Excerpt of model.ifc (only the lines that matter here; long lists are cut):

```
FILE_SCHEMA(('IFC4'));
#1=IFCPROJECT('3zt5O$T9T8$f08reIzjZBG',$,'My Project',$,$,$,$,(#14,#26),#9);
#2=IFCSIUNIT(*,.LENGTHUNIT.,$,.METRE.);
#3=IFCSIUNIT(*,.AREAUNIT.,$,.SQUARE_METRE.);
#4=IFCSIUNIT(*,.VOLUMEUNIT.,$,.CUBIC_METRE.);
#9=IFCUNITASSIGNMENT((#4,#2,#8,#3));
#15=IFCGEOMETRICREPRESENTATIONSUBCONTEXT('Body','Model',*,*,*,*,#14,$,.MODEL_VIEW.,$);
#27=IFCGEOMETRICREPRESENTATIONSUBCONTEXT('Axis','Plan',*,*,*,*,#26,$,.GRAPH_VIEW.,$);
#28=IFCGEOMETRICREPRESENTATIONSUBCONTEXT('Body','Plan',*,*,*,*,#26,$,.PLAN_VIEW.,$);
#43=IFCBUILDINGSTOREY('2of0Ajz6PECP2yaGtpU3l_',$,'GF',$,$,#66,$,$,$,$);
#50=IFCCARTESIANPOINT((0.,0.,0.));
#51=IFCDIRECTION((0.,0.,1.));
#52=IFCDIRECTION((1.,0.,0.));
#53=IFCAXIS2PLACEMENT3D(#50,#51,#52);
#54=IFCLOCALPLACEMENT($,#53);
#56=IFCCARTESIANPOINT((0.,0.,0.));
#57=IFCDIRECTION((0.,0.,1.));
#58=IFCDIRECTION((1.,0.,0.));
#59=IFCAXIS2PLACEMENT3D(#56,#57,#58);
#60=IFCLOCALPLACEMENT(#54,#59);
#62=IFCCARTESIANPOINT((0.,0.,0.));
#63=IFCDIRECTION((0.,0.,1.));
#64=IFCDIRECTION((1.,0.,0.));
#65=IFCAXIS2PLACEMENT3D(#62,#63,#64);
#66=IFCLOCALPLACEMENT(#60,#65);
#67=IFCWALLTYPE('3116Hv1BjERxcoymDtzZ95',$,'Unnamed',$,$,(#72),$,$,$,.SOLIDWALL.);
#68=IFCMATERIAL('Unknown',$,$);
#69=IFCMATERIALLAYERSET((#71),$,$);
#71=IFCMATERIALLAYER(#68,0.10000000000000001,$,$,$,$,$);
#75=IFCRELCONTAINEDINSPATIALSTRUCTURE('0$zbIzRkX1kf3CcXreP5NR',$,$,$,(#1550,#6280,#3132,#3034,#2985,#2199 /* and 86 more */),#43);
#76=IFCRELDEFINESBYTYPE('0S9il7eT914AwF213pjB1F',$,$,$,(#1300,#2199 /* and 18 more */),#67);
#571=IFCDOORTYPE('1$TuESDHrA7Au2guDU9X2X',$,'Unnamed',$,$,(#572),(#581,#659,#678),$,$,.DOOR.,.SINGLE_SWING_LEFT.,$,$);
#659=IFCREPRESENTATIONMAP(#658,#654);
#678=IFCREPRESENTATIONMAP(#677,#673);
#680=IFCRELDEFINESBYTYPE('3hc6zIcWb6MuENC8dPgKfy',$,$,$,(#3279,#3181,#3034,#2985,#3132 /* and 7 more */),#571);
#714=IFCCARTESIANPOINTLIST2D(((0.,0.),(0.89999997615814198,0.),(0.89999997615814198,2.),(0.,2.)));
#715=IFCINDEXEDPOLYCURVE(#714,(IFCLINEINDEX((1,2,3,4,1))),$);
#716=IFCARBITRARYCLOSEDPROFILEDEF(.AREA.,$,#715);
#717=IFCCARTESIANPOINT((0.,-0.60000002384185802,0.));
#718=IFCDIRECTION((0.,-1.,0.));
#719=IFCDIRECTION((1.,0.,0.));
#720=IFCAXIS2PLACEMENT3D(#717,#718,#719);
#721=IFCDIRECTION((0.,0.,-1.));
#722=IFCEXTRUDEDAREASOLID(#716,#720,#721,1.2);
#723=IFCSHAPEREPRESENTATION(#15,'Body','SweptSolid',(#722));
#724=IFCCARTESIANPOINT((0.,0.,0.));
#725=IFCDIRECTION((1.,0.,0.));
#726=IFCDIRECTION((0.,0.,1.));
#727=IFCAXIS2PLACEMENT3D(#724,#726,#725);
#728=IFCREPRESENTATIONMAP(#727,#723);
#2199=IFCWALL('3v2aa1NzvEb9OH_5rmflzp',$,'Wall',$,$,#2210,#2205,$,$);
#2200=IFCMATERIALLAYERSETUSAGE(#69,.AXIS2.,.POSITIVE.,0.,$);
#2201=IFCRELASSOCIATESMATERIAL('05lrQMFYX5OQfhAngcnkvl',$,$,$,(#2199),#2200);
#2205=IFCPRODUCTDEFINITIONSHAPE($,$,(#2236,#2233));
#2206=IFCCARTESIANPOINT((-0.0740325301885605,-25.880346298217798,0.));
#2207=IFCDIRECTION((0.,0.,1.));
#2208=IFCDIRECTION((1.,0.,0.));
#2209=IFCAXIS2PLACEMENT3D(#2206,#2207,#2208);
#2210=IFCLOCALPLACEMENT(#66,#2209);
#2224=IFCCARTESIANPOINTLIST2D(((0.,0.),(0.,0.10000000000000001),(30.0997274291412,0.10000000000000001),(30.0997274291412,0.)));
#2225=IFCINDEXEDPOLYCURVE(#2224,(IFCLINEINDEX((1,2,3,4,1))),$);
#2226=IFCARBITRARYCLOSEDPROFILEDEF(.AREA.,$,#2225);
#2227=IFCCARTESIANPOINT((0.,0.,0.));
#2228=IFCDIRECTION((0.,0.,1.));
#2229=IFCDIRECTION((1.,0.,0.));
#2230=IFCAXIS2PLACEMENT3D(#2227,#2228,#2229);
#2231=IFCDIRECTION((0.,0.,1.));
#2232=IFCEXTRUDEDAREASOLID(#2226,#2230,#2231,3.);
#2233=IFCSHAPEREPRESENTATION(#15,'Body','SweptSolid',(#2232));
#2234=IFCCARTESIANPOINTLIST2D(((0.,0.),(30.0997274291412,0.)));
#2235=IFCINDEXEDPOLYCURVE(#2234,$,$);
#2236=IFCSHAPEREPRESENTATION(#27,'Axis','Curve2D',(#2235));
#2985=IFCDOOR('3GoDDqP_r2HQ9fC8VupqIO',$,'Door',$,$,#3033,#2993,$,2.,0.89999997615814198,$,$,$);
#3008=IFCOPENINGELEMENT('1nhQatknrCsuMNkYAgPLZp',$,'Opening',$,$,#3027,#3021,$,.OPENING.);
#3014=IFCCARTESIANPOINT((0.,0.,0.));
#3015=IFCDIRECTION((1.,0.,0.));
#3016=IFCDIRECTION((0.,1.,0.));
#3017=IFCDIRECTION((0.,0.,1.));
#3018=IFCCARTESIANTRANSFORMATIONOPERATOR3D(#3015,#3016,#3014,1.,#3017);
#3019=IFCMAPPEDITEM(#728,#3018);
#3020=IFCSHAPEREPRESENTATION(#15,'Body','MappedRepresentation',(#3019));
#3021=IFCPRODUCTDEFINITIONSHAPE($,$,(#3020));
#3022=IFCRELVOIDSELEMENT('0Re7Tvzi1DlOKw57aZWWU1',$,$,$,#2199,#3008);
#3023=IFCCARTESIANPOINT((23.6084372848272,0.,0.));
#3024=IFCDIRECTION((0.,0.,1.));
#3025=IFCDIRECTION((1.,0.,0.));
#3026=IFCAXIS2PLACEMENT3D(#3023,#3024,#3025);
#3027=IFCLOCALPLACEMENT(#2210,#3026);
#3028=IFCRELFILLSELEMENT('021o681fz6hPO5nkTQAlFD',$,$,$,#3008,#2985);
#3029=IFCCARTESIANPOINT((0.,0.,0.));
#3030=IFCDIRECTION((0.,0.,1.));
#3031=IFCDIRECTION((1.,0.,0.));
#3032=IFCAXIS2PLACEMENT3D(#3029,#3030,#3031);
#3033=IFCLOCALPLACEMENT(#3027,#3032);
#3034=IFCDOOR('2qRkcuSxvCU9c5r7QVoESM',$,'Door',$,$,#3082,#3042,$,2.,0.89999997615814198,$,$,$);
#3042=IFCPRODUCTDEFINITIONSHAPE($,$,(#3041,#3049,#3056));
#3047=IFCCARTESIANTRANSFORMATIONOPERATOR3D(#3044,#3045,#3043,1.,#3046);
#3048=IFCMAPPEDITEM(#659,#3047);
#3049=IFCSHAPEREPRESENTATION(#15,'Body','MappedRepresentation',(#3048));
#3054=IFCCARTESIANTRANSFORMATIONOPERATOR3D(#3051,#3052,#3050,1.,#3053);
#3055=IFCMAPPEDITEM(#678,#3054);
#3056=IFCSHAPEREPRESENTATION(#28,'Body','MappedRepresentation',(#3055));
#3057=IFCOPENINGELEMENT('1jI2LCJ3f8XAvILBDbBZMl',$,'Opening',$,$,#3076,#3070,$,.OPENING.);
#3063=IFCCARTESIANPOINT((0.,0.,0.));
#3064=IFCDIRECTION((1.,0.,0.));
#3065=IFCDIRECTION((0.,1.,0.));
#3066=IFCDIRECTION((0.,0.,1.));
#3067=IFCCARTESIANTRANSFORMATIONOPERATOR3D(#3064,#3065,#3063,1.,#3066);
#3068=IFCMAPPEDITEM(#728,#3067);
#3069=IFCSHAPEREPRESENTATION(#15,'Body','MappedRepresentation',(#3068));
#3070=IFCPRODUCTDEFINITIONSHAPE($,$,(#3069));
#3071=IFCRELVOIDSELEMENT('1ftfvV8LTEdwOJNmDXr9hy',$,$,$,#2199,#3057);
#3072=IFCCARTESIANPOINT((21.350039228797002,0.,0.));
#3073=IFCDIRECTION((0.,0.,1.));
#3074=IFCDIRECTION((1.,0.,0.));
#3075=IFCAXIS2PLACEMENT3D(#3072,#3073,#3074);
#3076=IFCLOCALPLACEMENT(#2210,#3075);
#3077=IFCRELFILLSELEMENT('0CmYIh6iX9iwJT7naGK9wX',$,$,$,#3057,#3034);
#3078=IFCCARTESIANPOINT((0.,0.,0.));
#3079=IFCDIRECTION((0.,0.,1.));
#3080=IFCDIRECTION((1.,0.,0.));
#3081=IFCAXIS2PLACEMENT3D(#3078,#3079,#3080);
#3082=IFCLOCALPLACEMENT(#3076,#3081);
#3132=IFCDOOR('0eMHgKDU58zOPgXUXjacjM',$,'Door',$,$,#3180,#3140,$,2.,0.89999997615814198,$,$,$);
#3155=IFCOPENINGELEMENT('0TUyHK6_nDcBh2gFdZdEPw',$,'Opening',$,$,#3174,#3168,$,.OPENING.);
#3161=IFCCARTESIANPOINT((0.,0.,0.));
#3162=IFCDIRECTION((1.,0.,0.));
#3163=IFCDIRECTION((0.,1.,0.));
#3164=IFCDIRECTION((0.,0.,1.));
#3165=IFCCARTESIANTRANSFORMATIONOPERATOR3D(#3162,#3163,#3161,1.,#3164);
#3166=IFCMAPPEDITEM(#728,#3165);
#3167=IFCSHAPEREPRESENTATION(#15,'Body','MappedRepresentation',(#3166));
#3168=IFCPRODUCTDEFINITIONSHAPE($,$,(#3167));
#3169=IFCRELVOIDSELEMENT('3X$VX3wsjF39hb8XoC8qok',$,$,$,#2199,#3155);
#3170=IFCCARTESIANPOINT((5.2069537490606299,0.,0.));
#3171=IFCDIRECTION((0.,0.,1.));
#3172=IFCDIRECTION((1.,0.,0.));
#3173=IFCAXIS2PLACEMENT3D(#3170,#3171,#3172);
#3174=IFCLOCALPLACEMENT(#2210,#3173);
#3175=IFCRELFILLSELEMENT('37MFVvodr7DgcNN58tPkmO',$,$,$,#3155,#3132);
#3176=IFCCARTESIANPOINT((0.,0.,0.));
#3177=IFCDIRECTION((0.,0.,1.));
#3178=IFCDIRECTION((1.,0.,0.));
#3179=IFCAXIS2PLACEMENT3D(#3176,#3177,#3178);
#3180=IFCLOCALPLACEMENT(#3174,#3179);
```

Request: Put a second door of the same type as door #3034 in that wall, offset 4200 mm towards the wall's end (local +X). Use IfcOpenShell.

```python
import ifcopenshell
import ifcopenshell.api.feature
import ifcopenshell.api.geometry
import ifcopenshell.api.root
import ifcopenshell.geom
import ifcopenshell.util.element
import ifcopenshell.util.placement
import ifcopenshell.util.shape
import ifcopenshell.util.unit

model = ifcopenshell.open("model.ifc")
unit_scale = ifcopenshell.util.unit.calculate_unit_scale(model)
settings = ifcopenshell.geom.settings()


def volume(element):
    """Net volume in cubic metres, openings subtracted."""
    shape = ifcopenshell.geom.create_shape(settings, element)
    return ifcopenshell.util.shape.get_volume(shape.geometry)


door = model.by_guid("2qRkcuSxvCU9c5r7QVoESM")
opening = door.FillsVoids[0].RelatingOpeningElement
wall = opening.VoidsElements[0].RelatingBuildingElement
before = volume(wall)
shift = ifcopenshell.util.placement.get_local_placement(wall.ObjectPlacement)[:3, 0] * 4.2 / unit_scale

# copy_class copies the void relationship, type, container and properties, but no geometry.
new_opening = ifcopenshell.api.root.copy_class(model, product=opening)
new_opening.Representation = ifcopenshell.util.element.copy_deep(
    model, opening.Representation, exclude=["IfcGeometricRepresentationContext", "IfcRepresentationMap"]
)
new_door = ifcopenshell.api.root.copy_class(model, product=door)
new_door.Representation = ifcopenshell.util.element.copy_deep(
    model, door.Representation, exclude=["IfcGeometricRepresentationContext", "IfcRepresentationMap"]
)
ifcopenshell.api.feature.add_filling(model, opening=new_opening, element=new_door)

for old, new in ((opening, new_opening), (door, new_door)):
    matrix = ifcopenshell.util.placement.get_local_placement(old.ObjectPlacement)
    matrix[:3, 3] += shift
    ifcopenshell.api.geometry.edit_object_placement(model, product=new, matrix=matrix, is_si=False)

after = volume(wall)

print(f"wall volume {before:.3f} -> {after:.3f} m3")

model.write("model_edited.ifc")
```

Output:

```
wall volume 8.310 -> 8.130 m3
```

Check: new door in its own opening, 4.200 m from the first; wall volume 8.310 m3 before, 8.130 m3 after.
